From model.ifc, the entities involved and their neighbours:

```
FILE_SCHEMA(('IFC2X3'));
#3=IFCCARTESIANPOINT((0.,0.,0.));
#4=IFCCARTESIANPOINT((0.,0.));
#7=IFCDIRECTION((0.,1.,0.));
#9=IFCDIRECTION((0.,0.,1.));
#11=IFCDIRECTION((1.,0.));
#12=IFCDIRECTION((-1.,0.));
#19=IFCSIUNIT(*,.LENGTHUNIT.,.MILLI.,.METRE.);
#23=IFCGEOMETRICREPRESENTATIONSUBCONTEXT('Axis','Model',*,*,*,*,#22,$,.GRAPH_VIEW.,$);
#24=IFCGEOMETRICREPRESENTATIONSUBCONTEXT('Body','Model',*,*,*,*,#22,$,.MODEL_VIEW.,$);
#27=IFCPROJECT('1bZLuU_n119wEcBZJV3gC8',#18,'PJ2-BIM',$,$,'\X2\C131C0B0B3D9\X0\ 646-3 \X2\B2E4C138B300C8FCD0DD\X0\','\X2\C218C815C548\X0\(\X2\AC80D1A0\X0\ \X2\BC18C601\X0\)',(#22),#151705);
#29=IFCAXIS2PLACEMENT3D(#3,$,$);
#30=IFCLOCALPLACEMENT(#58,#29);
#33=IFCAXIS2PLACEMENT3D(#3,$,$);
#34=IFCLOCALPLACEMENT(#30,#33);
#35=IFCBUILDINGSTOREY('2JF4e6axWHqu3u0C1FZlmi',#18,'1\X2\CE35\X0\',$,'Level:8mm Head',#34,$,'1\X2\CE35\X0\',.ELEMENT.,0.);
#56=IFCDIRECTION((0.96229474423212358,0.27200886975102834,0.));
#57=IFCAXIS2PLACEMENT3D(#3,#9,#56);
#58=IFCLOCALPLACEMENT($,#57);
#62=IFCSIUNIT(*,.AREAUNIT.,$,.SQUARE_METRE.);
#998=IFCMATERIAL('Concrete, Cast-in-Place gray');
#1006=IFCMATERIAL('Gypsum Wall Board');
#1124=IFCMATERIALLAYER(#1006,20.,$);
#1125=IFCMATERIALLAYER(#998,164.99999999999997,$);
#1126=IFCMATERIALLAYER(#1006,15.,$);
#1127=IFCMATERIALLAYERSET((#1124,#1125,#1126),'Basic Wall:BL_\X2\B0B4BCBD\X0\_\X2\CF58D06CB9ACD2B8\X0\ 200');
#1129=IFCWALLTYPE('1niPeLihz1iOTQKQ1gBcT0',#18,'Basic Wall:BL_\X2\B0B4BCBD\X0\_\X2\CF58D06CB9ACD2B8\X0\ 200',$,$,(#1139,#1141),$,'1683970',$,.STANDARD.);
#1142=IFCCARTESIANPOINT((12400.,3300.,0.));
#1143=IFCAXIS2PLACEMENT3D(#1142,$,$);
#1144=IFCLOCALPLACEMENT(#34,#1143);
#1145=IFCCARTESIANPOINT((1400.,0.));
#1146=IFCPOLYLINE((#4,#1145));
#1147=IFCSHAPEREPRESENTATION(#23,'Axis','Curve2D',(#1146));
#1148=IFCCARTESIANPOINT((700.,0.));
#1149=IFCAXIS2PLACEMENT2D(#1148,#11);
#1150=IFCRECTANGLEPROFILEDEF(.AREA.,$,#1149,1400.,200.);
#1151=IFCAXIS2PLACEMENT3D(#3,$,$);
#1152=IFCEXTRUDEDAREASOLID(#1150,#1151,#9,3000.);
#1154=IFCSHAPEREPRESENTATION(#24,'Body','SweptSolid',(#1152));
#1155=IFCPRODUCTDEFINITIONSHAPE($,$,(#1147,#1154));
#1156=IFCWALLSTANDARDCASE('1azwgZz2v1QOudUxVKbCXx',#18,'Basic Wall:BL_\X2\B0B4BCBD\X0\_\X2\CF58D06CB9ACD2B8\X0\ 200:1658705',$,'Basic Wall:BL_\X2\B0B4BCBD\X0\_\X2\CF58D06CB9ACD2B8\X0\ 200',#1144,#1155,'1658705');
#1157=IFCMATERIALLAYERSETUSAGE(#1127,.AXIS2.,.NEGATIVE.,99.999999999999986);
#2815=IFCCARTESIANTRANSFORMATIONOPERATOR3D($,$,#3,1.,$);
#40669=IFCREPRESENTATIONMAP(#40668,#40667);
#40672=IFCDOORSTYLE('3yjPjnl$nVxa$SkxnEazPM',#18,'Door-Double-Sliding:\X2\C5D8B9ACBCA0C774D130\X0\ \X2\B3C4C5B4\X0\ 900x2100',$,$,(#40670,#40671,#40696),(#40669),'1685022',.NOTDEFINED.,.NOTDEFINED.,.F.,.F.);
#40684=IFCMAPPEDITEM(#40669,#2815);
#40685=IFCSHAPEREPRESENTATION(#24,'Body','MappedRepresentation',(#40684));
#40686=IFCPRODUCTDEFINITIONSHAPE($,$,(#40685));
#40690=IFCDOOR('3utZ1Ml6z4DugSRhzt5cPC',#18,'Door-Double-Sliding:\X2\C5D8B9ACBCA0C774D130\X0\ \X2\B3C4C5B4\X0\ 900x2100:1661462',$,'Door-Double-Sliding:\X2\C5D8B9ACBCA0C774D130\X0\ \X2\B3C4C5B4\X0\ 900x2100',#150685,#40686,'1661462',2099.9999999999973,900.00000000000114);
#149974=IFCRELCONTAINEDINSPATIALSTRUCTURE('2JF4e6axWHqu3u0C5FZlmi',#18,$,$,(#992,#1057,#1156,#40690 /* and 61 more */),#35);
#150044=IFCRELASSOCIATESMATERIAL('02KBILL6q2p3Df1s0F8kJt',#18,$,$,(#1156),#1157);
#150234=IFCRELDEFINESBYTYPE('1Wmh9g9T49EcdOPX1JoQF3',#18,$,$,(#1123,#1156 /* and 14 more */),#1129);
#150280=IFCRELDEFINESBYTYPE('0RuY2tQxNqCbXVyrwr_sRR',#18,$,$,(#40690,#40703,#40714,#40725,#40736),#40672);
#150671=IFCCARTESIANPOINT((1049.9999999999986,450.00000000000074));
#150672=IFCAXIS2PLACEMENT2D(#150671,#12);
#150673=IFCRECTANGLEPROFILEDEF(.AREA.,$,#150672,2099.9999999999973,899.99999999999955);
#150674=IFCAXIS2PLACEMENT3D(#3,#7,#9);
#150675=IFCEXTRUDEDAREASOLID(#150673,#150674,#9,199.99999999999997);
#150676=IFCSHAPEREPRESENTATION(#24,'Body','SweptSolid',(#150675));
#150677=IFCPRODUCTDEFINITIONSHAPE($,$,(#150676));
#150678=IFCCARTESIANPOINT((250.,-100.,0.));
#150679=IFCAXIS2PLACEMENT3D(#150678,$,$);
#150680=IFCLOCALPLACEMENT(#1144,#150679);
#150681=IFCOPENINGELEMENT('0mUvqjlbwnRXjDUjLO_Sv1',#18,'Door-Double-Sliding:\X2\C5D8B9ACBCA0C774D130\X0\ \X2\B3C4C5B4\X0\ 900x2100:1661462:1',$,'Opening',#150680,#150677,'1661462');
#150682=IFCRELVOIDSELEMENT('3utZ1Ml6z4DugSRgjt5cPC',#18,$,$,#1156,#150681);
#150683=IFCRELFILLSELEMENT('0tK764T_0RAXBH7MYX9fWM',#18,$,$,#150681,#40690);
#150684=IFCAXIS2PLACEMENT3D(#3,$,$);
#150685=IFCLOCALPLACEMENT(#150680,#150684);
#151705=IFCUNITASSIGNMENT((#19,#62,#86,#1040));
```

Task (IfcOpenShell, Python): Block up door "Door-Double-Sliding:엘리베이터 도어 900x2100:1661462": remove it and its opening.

```python
import ifcopenshell
import ifcopenshell.api.feature
import ifcopenshell.api.root
import ifcopenshell.geom
import ifcopenshell.util.shape

model = ifcopenshell.open("model.ifc")
settings = ifcopenshell.geom.settings()


def volume(element):
    """Net volume in cubic metres, openings subtracted."""
    shape = ifcopenshell.geom.create_shape(settings, element)
    return ifcopenshell.util.shape.get_volume(shape.geometry)


door = model.by_guid("3utZ1Ml6z4DugSRhzt5cPC")
opening = door.FillsVoids[0].RelatingOpeningElement
wall = opening.VoidsElements[0].RelatingBuildingElement
before = volume(wall)

ifcopenshell.api.root.remove_product(model, product=door)
ifcopenshell.api.feature.remove_feature(model, feature=opening)

after = volume(wall)

print(f"wall volume {before:.3f} -> {after:.3f} m3")

model.write("model_edited.ifc")
```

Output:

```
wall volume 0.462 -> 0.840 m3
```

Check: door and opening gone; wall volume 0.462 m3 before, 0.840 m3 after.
